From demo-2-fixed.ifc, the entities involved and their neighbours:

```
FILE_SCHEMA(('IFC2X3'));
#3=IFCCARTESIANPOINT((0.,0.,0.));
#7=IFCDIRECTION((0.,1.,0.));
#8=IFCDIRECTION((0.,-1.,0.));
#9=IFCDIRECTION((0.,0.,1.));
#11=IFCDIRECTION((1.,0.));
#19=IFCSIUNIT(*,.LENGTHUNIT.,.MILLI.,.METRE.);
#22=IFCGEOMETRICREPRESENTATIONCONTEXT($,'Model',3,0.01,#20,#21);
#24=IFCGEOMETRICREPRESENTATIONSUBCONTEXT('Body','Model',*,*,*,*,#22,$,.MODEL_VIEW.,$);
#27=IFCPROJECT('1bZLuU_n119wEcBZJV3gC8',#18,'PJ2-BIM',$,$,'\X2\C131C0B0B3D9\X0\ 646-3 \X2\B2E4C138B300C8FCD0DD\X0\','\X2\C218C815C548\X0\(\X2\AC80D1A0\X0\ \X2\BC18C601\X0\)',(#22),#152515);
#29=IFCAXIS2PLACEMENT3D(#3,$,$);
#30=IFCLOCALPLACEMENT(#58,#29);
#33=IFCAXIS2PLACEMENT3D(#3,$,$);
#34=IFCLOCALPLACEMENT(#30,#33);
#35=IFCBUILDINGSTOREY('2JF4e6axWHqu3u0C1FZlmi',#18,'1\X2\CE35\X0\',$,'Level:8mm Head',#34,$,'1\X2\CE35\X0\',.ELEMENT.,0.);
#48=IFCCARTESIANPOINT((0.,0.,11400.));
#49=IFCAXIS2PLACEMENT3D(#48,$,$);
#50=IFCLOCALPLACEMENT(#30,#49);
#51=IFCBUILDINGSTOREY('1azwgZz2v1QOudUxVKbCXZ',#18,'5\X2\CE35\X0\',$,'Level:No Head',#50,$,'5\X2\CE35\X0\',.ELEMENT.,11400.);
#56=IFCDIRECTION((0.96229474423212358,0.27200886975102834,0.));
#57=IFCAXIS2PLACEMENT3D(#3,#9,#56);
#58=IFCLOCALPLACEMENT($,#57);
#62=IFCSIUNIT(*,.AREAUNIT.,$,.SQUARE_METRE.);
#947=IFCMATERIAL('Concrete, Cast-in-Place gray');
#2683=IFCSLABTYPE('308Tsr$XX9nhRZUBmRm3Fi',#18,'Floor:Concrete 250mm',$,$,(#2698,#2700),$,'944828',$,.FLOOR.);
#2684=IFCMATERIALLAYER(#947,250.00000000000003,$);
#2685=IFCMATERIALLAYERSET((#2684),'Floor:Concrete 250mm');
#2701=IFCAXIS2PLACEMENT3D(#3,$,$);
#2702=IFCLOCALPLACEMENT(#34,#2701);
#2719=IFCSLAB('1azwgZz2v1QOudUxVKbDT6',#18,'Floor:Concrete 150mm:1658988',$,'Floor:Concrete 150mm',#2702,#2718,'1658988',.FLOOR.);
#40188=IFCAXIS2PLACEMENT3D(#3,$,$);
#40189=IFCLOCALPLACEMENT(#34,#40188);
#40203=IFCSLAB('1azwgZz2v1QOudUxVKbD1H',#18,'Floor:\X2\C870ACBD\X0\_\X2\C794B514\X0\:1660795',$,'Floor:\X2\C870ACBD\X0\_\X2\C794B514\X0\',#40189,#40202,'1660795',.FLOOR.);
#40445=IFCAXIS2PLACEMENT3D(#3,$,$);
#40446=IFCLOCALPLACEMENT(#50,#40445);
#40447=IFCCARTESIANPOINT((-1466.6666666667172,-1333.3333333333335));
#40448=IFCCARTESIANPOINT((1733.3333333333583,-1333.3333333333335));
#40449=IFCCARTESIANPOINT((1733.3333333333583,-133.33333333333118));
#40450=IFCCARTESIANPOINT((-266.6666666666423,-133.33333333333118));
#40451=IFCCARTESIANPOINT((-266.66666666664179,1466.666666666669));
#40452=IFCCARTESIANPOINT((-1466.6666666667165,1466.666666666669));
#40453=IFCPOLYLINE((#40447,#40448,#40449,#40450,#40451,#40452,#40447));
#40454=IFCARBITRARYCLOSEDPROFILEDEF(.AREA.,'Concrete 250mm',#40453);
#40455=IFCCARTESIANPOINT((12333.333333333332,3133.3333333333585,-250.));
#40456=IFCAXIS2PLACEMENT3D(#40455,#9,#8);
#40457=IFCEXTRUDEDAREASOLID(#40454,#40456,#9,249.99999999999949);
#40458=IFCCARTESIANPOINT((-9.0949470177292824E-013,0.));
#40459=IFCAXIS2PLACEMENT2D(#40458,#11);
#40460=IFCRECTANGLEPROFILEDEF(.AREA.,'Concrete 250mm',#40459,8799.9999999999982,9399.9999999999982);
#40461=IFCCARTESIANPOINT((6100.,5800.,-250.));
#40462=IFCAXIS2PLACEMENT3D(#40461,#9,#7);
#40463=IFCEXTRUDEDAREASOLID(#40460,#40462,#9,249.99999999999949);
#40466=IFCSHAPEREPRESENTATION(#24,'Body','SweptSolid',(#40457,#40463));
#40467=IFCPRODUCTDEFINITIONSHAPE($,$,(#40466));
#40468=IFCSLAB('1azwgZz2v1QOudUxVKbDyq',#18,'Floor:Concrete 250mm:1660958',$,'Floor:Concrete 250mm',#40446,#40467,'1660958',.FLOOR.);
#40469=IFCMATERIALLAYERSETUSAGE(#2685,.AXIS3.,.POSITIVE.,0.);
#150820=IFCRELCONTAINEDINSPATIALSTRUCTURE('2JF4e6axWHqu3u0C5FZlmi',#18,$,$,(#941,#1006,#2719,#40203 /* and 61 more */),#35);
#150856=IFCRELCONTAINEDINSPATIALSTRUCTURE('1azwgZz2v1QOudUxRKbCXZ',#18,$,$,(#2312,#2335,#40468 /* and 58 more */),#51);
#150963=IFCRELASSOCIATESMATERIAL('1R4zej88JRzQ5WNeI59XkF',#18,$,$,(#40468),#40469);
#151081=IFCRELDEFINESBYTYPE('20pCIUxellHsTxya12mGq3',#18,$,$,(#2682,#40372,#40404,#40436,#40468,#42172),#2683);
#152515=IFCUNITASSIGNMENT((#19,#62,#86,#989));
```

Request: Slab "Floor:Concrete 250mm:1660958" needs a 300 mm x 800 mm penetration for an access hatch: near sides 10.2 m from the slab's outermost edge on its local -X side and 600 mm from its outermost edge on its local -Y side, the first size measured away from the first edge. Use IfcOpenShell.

```python
import numpy as np
import ifcopenshell
import ifcopenshell.api.feature
import ifcopenshell.api.geometry
import ifcopenshell.api.root
import ifcopenshell.geom
import ifcopenshell.util.placement
import ifcopenshell.util.representation
import ifcopenshell.util.shape
import ifcopenshell.util.unit

model = ifcopenshell.open("demo-2-fixed.ifc")
unit_scale = ifcopenshell.util.unit.calculate_unit_scale(model)
settings = ifcopenshell.geom.settings()


def volume(element):
    """Net volume in cubic metres, openings subtracted."""
    shape = ifcopenshell.geom.create_shape(settings, element)
    return ifcopenshell.util.shape.get_volume(shape.geometry)


slab = model.by_guid("1azwgZz2v1QOudUxVKbDyq")
before = volume(slab)

# Extent in the slab's own axes, in metres. The edges named are its -X and -Y sides.
slab_shape = ifcopenshell.geom.create_shape(settings, slab)
vertices = ifcopenshell.util.shape.get_vertices(slab_shape.geometry)
x_min, y_min, bottom = vertices.min(axis=0)
top = vertices[:, 2].max()

opening = ifcopenshell.api.root.create_entity(model, ifc_class="IfcOpeningElement", name="Access hatch opening")
context = ifcopenshell.util.representation.get_context(model, "Model", "Body", "MODEL_VIEW")
width, depth = 0.3, 0.8
outline = [(0.0, 0.0), (width, 0.0), (width, depth), (0.0, depth), (0.0, 0.0)]
# Overshoot both faces by 50 mm so the cut is clean.
shape = ifcopenshell.api.geometry.add_slab_representation(
    model, context=context, depth=top - bottom + 0.1, polyline=outline
)
ifcopenshell.api.geometry.assign_representation(model, product=opening, representation=shape)

matrix = ifcopenshell.util.placement.get_local_placement(slab.ObjectPlacement)
matrix[:, 3] = matrix @ np.append(np.array([x_min + 10.2, y_min + 0.6, bottom - 0.05]) / unit_scale, 1.0)
ifcopenshell.api.geometry.edit_object_placement(model, product=opening, matrix=matrix, is_si=False)
ifcopenshell.api.feature.add_feature(model, feature=opening, element=slab)

after = volume(slab)

print(f"slab volume {before:.3f} -> {after:.3f} m3")

model.write("demo-2-fixed_updated.ifc")
```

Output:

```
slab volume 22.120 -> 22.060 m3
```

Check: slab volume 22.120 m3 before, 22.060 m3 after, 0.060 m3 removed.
